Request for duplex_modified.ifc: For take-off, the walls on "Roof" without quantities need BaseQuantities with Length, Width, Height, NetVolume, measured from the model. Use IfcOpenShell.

First a look at what the model holds.

```python
import ifcopenshell
import ifcopenshell.util.element
import ifcopenshell.util.unit

model = ifcopenshell.open("duplex_modified.ifc")
print(model.schema)
for unit_type in ("LENGTHUNIT", "AREAUNIT", "VOLUMEUNIT"):
    print(unit_type, ifcopenshell.util.unit.calculate_unit_scale(model, unit_type))
storey = next(s for s in model.by_type("IfcBuildingStorey") if s.Name == "Roof")
walls = [e for e in ifcopenshell.util.element.get_decomposition(storey) if e.is_a("IfcWall")]
for e in sorted(walls, key=lambda e: e.id()):
    print(e.id(), e.is_a(), e.Name, list(ifcopenshell.util.element.get_psets(e, qtos_only=True)), sep=" | ")
```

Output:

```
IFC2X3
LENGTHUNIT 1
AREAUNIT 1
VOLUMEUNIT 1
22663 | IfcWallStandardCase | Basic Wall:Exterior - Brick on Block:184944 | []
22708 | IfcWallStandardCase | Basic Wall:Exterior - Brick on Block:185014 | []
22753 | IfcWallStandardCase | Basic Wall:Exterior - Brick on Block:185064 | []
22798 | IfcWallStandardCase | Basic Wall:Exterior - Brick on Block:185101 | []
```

```python
import ifcopenshell
import ifcopenshell.api.pset
import ifcopenshell.geom
import ifcopenshell.util.element
import ifcopenshell.util.shape
import ifcopenshell.util.unit

model = ifcopenshell.open("duplex_modified.ifc")
unit_scale = ifcopenshell.util.unit.calculate_unit_scale(model)
volume_scale = ifcopenshell.util.unit.calculate_unit_scale(model, "VOLUMEUNIT")
settings = ifcopenshell.geom.settings()

storey = next(s for s in model.by_type("IfcBuildingStorey") if s.Name == "Roof")
walls = [e for e in ifcopenshell.util.element.get_decomposition(storey) if e.is_a("IfcWall")]

for e in sorted(walls, key=lambda e: e.id()):
    if ifcopenshell.util.element.get_psets(e, qtos_only=True, should_inherit=False):
        continue
    # Geometry comes back in metres, in the element's own axes.
    shape = ifcopenshell.geom.create_shape(settings, e)
    values = {
        "Length": ifcopenshell.util.shape.get_x(shape.geometry) / unit_scale,
        "Width": ifcopenshell.util.shape.get_y(shape.geometry) / unit_scale,
        "Height": ifcopenshell.util.shape.get_z(shape.geometry) / unit_scale,
        "NetVolume": ifcopenshell.util.shape.get_volume(shape.geometry) / volume_scale,
    }
    qto = ifcopenshell.api.pset.add_qto(model, product=e, name="BaseQuantities")
    ifcopenshell.api.pset.edit_qto(model, qto=qto, properties=values)
    print(e.id(), {k: round(v, 3) for k, v in values.items()})

model.write("duplex_modified_updated.ifc")
```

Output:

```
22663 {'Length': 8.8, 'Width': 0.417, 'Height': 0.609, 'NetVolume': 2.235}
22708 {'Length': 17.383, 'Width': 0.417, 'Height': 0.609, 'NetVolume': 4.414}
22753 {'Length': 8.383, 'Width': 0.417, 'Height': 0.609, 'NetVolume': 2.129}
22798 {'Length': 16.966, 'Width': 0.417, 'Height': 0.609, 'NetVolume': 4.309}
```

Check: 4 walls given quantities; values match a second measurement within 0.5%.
